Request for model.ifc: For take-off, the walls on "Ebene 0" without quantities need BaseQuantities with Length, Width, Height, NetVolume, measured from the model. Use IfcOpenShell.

First a look at what the model holds.

```python
import ifcopenshell
import ifcopenshell.util.element
import ifcopenshell.util.unit

model = ifcopenshell.open("model.ifc")
print(model.schema)
for unit_type in ("LENGTHUNIT", "AREAUNIT", "VOLUMEUNIT"):
    print(unit_type, ifcopenshell.util.unit.calculate_unit_scale(model, unit_type))
storey = next(s for s in model.by_type("IfcBuildingStorey") if s.Name == "Ebene 0")
walls = [e for e in ifcopenshell.util.element.get_decomposition(storey) if e.is_a("IfcWall")]
for e in sorted(walls, key=lambda e: e.id()):
    print(e.id(), e.is_a(), e.Name, list(ifcopenshell.util.element.get_psets(e, qtos_only=True)), sep=" | ")
```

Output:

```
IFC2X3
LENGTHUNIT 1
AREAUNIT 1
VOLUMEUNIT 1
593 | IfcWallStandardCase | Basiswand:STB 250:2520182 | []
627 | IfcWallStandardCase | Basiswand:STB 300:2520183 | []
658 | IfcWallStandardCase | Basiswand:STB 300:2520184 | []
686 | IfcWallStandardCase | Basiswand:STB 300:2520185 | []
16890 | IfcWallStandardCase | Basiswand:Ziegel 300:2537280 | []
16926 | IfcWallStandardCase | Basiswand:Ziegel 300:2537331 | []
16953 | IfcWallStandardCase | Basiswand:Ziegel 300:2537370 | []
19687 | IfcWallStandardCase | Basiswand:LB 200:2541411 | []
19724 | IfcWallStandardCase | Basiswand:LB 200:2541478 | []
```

```python
import ifcopenshell
import ifcopenshell.api.pset
import ifcopenshell.geom
import ifcopenshell.util.element
import ifcopenshell.util.shape
import ifcopenshell.util.unit

model = ifcopenshell.open("model.ifc")
unit_scale = ifcopenshell.util.unit.calculate_unit_scale(model)
volume_scale = ifcopenshell.util.unit.calculate_unit_scale(model, "VOLUMEUNIT")
settings = ifcopenshell.geom.settings()

storey = next(s for s in model.by_type("IfcBuildingStorey") if s.Name == "Ebene 0")
walls = [e for e in ifcopenshell.util.element.get_decomposition(storey) if e.is_a("IfcWall")]

for e in sorted(walls, key=lambda e: e.id()):
    if ifcopenshell.util.element.get_psets(e, qtos_only=True, should_inherit=False):
        continue
    # Geometry comes back in metres, in the element's own axes.
    shape = ifcopenshell.geom.create_shape(settings, e)
    values = {
        "Length": ifcopenshell.util.shape.get_x(shape.geometry) / unit_scale,
        "Width": ifcopenshell.util.shape.get_y(shape.geometry) / unit_scale,
        "Height": ifcopenshell.util.shape.get_z(shape.geometry) / unit_scale,
        "NetVolume": ifcopenshell.util.shape.get_volume(shape.geometry) / volume_scale,
    }
    qto = ifcopenshell.api.pset.add_qto(model, product=e, name="BaseQuantities")
    ifcopenshell.api.pset.edit_qto(model, qto=qto, properties=values)
    print(e.id(), {k: round(v, 3) for k, v in values.items()})

model.write("model_edited.ifc")
```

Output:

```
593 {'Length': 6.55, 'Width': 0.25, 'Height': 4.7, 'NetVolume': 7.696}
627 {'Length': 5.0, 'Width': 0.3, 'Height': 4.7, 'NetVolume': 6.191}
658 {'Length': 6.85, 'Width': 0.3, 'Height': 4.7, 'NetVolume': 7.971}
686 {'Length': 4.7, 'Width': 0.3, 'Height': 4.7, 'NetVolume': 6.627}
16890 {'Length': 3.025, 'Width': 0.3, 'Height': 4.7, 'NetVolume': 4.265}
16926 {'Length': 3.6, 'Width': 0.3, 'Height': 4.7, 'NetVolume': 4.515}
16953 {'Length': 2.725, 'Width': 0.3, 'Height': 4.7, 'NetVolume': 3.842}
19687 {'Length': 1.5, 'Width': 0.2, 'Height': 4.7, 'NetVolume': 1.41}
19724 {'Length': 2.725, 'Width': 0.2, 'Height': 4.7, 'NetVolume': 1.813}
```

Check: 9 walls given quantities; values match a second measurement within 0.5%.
